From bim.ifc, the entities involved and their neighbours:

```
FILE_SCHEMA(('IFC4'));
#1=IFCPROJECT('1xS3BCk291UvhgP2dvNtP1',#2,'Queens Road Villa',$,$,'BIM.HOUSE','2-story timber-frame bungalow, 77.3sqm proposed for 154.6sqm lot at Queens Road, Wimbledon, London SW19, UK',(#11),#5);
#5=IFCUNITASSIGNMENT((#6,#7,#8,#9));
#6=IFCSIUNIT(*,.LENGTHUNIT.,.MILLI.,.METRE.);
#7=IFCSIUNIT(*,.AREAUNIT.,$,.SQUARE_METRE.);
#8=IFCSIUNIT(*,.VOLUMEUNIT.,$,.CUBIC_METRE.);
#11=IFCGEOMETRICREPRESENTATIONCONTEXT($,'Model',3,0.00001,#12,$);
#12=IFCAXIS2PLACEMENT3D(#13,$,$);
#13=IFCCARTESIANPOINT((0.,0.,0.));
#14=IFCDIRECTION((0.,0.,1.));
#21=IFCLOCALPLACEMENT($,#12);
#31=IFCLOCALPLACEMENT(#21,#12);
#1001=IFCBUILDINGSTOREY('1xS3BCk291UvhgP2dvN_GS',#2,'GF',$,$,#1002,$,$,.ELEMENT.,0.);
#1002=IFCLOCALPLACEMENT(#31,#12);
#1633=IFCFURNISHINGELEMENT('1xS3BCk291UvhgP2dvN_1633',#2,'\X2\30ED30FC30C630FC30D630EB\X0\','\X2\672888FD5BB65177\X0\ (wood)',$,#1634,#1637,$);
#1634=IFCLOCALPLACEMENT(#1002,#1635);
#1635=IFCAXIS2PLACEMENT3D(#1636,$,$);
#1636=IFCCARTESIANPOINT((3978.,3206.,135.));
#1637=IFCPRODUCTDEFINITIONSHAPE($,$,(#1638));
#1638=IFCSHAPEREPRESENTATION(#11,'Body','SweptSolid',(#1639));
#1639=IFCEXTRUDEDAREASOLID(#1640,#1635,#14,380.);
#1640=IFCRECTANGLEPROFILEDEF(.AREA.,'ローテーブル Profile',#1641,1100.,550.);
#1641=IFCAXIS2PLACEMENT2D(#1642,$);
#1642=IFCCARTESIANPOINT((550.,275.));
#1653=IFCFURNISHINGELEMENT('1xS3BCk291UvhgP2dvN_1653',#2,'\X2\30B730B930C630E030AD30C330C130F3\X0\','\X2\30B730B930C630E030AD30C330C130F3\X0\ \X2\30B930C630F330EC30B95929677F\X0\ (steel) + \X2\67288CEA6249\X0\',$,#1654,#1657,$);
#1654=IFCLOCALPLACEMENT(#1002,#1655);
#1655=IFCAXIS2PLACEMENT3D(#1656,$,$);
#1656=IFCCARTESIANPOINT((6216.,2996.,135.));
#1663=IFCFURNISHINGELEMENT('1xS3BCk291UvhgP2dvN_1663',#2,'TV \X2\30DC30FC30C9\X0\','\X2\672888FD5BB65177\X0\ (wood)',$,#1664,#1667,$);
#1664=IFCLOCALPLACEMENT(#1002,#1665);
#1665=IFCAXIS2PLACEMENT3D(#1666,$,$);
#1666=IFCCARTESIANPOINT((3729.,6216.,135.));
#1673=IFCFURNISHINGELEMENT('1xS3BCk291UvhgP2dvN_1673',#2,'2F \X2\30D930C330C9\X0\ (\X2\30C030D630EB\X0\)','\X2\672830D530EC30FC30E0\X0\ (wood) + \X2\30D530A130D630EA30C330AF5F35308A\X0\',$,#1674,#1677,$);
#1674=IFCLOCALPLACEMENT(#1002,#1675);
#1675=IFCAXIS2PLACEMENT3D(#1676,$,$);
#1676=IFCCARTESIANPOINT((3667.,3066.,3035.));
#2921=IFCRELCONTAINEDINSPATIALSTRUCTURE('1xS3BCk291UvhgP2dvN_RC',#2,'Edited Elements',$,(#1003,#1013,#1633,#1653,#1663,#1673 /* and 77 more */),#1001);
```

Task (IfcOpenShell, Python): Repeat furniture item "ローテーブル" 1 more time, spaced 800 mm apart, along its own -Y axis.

```python
import ifcopenshell
import ifcopenshell.api.geometry
import ifcopenshell.api.root
import ifcopenshell.util.element
import ifcopenshell.util.placement
import ifcopenshell.util.unit

model = ifcopenshell.open("bim.ifc")
unit_scale = ifcopenshell.util.unit.calculate_unit_scale(model)


def reuse_history(source, copy):
    """copy_class also copies each property set's owner history, people and application; keep the originals."""
    for rel in copy.IsDefinedBy:
        if rel.is_a("IfcRelDefinesByProperties") and (history := rel.RelatingPropertyDefinition.OwnerHistory):
            rel.RelatingPropertyDefinition.OwnerHistory = source.OwnerHistory
            ifcopenshell.util.element.remove_deep2(model, history)


source = model.by_guid("1xS3BCk291UvhgP2dvN_1633")
base = ifcopenshell.util.placement.get_local_placement(source.ObjectPlacement)
step = -base[:3, 1] * 0.8 / unit_scale

for i in range(1, 2):
    copy = ifcopenshell.api.root.copy_class(model, product=source)
    copy.Representation = ifcopenshell.util.element.copy_deep(
        model, source.Representation, exclude=["IfcGeometricRepresentationContext", "IfcRepresentationMap"]
    )
    reuse_history(source, copy)
    matrix = base.copy()
    matrix[:3, 3] += i * step
    print("added at", matrix[:3, 3].round(3) + 0.0)
    ifcopenshell.api.geometry.edit_object_placement(model, product=copy, matrix=matrix, is_si=False)

model.write("bim_rev.ifc")
```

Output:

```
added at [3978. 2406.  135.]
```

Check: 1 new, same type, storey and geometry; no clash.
